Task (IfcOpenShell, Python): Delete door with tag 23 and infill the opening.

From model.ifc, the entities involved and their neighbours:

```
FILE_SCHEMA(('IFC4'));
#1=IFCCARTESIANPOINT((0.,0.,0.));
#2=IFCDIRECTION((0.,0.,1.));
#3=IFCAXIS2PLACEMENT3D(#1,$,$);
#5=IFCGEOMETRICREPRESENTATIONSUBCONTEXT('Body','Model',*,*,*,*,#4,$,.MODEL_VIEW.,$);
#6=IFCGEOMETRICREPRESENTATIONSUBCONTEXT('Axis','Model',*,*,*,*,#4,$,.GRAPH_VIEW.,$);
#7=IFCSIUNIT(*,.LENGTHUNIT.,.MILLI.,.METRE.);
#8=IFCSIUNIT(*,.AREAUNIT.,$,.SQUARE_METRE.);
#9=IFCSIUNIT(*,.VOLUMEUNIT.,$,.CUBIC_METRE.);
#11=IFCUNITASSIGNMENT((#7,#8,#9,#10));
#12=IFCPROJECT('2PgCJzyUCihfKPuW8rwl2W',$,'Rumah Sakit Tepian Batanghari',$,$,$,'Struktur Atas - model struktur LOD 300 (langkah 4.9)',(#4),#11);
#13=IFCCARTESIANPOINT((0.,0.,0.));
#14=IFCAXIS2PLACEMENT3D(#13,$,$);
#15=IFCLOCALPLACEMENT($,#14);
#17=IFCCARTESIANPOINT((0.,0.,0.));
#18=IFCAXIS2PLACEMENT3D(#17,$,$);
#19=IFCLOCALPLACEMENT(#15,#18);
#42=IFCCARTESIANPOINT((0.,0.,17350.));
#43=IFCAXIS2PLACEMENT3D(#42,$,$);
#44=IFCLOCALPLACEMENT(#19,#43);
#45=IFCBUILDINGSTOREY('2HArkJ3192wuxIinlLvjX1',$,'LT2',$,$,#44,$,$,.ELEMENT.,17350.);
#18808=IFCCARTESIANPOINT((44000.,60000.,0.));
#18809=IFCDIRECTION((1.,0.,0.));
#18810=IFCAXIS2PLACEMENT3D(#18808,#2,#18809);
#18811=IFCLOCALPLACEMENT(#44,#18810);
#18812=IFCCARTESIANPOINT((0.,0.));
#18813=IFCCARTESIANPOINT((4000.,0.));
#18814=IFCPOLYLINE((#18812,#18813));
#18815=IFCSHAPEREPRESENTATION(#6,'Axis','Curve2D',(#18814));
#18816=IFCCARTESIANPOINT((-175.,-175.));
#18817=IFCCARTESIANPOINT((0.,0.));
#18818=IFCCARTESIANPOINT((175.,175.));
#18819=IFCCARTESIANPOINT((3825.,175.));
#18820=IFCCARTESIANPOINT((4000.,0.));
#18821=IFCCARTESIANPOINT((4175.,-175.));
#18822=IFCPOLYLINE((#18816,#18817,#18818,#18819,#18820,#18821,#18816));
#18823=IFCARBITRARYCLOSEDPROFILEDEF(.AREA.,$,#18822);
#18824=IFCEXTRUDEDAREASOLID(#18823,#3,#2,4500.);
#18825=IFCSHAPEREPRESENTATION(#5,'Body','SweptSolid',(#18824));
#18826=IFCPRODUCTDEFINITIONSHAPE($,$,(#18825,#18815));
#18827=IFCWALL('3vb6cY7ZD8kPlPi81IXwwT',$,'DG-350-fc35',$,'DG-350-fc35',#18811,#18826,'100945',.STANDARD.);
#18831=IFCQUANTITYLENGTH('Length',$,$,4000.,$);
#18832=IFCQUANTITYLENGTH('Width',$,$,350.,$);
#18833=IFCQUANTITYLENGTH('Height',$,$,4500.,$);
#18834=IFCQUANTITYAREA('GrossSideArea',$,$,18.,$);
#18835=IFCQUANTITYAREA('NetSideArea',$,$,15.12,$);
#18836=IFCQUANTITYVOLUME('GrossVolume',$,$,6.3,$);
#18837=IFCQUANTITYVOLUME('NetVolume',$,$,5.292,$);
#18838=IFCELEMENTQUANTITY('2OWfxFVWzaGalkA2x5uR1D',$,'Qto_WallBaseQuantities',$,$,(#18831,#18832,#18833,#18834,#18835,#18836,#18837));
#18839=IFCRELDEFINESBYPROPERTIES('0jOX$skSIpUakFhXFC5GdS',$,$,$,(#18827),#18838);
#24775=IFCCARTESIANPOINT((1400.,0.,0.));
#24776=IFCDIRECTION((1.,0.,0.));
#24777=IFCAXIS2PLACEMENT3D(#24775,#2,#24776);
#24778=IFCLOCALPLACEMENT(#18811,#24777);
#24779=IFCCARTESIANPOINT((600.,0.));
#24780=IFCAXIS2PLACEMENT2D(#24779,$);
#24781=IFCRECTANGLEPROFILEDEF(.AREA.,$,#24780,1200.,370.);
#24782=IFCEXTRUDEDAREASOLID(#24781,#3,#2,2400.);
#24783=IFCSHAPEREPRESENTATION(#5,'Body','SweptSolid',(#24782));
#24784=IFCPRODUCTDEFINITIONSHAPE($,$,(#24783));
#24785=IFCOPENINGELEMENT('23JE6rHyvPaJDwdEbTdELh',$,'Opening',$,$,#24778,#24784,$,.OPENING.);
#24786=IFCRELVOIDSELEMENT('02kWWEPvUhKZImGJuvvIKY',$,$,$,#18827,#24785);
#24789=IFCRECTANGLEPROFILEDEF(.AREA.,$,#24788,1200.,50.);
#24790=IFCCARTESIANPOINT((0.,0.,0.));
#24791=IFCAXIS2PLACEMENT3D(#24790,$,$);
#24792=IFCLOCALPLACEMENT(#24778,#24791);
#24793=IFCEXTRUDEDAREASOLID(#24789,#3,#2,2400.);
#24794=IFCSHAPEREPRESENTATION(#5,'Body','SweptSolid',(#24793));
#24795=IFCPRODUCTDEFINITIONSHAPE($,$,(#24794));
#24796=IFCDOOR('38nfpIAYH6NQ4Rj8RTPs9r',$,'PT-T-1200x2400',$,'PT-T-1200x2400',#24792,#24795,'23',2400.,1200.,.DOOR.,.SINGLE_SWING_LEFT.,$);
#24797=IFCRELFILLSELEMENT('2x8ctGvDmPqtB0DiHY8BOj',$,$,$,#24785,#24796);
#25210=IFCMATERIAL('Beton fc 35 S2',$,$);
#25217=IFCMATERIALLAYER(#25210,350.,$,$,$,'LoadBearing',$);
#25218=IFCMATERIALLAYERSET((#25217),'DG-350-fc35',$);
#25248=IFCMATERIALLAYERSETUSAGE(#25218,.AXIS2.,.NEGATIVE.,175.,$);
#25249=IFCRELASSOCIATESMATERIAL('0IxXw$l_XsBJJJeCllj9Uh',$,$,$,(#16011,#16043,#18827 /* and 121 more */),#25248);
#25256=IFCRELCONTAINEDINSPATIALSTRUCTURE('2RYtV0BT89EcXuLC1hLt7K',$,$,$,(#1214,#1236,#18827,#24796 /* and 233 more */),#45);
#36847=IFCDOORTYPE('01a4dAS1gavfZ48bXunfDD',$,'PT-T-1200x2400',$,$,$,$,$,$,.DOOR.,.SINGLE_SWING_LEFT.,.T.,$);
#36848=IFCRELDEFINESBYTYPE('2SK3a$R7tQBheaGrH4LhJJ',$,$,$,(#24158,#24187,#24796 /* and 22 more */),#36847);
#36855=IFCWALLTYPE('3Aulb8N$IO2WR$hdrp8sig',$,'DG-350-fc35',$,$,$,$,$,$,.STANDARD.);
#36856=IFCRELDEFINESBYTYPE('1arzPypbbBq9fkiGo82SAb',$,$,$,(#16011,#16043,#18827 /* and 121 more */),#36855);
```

```python
import ifcopenshell
import ifcopenshell.api.feature
import ifcopenshell.api.pset
import ifcopenshell.api.root
import ifcopenshell.geom
import ifcopenshell.util.element
import ifcopenshell.util.shape
import ifcopenshell.util.unit

model = ifcopenshell.open("model.ifc")
area_scale = ifcopenshell.util.unit.calculate_unit_scale(model, "AREAUNIT")
volume_scale = ifcopenshell.util.unit.calculate_unit_scale(model, "VOLUMEUNIT")
settings = ifcopenshell.geom.settings()


def volume(element):
    """Net volume in cubic metres, openings subtracted."""
    shape = ifcopenshell.geom.create_shape(settings, element)
    return ifcopenshell.util.shape.get_volume(shape.geometry)


door = model.by_id(24796)
opening = door.FillsVoids[0].RelatingOpeningElement
wall = opening.VoidsElements[0].RelatingBuildingElement
before = volume(wall)

ifcopenshell.api.root.remove_product(model, product=door)
ifcopenshell.api.feature.remove_feature(model, feature=opening)

after = volume(wall)
thickness = 0.35  # wall thickness in metres

# Update the wall's stored quantities.
qto = model.by_id(ifcopenshell.util.element.get_pset(wall, "Qto_WallBaseQuantities", should_inherit=False)["id"])
ifcopenshell.api.pset.edit_qto(model, qto=qto, properties={
    "NetSideArea": after / thickness / area_scale,
    "NetVolume": after / volume_scale,
})

print(f"wall volume {before:.3f} -> {after:.3f} m3")

model.write("model_updated.ifc")
```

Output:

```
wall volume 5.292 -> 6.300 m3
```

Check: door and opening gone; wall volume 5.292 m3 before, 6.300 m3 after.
